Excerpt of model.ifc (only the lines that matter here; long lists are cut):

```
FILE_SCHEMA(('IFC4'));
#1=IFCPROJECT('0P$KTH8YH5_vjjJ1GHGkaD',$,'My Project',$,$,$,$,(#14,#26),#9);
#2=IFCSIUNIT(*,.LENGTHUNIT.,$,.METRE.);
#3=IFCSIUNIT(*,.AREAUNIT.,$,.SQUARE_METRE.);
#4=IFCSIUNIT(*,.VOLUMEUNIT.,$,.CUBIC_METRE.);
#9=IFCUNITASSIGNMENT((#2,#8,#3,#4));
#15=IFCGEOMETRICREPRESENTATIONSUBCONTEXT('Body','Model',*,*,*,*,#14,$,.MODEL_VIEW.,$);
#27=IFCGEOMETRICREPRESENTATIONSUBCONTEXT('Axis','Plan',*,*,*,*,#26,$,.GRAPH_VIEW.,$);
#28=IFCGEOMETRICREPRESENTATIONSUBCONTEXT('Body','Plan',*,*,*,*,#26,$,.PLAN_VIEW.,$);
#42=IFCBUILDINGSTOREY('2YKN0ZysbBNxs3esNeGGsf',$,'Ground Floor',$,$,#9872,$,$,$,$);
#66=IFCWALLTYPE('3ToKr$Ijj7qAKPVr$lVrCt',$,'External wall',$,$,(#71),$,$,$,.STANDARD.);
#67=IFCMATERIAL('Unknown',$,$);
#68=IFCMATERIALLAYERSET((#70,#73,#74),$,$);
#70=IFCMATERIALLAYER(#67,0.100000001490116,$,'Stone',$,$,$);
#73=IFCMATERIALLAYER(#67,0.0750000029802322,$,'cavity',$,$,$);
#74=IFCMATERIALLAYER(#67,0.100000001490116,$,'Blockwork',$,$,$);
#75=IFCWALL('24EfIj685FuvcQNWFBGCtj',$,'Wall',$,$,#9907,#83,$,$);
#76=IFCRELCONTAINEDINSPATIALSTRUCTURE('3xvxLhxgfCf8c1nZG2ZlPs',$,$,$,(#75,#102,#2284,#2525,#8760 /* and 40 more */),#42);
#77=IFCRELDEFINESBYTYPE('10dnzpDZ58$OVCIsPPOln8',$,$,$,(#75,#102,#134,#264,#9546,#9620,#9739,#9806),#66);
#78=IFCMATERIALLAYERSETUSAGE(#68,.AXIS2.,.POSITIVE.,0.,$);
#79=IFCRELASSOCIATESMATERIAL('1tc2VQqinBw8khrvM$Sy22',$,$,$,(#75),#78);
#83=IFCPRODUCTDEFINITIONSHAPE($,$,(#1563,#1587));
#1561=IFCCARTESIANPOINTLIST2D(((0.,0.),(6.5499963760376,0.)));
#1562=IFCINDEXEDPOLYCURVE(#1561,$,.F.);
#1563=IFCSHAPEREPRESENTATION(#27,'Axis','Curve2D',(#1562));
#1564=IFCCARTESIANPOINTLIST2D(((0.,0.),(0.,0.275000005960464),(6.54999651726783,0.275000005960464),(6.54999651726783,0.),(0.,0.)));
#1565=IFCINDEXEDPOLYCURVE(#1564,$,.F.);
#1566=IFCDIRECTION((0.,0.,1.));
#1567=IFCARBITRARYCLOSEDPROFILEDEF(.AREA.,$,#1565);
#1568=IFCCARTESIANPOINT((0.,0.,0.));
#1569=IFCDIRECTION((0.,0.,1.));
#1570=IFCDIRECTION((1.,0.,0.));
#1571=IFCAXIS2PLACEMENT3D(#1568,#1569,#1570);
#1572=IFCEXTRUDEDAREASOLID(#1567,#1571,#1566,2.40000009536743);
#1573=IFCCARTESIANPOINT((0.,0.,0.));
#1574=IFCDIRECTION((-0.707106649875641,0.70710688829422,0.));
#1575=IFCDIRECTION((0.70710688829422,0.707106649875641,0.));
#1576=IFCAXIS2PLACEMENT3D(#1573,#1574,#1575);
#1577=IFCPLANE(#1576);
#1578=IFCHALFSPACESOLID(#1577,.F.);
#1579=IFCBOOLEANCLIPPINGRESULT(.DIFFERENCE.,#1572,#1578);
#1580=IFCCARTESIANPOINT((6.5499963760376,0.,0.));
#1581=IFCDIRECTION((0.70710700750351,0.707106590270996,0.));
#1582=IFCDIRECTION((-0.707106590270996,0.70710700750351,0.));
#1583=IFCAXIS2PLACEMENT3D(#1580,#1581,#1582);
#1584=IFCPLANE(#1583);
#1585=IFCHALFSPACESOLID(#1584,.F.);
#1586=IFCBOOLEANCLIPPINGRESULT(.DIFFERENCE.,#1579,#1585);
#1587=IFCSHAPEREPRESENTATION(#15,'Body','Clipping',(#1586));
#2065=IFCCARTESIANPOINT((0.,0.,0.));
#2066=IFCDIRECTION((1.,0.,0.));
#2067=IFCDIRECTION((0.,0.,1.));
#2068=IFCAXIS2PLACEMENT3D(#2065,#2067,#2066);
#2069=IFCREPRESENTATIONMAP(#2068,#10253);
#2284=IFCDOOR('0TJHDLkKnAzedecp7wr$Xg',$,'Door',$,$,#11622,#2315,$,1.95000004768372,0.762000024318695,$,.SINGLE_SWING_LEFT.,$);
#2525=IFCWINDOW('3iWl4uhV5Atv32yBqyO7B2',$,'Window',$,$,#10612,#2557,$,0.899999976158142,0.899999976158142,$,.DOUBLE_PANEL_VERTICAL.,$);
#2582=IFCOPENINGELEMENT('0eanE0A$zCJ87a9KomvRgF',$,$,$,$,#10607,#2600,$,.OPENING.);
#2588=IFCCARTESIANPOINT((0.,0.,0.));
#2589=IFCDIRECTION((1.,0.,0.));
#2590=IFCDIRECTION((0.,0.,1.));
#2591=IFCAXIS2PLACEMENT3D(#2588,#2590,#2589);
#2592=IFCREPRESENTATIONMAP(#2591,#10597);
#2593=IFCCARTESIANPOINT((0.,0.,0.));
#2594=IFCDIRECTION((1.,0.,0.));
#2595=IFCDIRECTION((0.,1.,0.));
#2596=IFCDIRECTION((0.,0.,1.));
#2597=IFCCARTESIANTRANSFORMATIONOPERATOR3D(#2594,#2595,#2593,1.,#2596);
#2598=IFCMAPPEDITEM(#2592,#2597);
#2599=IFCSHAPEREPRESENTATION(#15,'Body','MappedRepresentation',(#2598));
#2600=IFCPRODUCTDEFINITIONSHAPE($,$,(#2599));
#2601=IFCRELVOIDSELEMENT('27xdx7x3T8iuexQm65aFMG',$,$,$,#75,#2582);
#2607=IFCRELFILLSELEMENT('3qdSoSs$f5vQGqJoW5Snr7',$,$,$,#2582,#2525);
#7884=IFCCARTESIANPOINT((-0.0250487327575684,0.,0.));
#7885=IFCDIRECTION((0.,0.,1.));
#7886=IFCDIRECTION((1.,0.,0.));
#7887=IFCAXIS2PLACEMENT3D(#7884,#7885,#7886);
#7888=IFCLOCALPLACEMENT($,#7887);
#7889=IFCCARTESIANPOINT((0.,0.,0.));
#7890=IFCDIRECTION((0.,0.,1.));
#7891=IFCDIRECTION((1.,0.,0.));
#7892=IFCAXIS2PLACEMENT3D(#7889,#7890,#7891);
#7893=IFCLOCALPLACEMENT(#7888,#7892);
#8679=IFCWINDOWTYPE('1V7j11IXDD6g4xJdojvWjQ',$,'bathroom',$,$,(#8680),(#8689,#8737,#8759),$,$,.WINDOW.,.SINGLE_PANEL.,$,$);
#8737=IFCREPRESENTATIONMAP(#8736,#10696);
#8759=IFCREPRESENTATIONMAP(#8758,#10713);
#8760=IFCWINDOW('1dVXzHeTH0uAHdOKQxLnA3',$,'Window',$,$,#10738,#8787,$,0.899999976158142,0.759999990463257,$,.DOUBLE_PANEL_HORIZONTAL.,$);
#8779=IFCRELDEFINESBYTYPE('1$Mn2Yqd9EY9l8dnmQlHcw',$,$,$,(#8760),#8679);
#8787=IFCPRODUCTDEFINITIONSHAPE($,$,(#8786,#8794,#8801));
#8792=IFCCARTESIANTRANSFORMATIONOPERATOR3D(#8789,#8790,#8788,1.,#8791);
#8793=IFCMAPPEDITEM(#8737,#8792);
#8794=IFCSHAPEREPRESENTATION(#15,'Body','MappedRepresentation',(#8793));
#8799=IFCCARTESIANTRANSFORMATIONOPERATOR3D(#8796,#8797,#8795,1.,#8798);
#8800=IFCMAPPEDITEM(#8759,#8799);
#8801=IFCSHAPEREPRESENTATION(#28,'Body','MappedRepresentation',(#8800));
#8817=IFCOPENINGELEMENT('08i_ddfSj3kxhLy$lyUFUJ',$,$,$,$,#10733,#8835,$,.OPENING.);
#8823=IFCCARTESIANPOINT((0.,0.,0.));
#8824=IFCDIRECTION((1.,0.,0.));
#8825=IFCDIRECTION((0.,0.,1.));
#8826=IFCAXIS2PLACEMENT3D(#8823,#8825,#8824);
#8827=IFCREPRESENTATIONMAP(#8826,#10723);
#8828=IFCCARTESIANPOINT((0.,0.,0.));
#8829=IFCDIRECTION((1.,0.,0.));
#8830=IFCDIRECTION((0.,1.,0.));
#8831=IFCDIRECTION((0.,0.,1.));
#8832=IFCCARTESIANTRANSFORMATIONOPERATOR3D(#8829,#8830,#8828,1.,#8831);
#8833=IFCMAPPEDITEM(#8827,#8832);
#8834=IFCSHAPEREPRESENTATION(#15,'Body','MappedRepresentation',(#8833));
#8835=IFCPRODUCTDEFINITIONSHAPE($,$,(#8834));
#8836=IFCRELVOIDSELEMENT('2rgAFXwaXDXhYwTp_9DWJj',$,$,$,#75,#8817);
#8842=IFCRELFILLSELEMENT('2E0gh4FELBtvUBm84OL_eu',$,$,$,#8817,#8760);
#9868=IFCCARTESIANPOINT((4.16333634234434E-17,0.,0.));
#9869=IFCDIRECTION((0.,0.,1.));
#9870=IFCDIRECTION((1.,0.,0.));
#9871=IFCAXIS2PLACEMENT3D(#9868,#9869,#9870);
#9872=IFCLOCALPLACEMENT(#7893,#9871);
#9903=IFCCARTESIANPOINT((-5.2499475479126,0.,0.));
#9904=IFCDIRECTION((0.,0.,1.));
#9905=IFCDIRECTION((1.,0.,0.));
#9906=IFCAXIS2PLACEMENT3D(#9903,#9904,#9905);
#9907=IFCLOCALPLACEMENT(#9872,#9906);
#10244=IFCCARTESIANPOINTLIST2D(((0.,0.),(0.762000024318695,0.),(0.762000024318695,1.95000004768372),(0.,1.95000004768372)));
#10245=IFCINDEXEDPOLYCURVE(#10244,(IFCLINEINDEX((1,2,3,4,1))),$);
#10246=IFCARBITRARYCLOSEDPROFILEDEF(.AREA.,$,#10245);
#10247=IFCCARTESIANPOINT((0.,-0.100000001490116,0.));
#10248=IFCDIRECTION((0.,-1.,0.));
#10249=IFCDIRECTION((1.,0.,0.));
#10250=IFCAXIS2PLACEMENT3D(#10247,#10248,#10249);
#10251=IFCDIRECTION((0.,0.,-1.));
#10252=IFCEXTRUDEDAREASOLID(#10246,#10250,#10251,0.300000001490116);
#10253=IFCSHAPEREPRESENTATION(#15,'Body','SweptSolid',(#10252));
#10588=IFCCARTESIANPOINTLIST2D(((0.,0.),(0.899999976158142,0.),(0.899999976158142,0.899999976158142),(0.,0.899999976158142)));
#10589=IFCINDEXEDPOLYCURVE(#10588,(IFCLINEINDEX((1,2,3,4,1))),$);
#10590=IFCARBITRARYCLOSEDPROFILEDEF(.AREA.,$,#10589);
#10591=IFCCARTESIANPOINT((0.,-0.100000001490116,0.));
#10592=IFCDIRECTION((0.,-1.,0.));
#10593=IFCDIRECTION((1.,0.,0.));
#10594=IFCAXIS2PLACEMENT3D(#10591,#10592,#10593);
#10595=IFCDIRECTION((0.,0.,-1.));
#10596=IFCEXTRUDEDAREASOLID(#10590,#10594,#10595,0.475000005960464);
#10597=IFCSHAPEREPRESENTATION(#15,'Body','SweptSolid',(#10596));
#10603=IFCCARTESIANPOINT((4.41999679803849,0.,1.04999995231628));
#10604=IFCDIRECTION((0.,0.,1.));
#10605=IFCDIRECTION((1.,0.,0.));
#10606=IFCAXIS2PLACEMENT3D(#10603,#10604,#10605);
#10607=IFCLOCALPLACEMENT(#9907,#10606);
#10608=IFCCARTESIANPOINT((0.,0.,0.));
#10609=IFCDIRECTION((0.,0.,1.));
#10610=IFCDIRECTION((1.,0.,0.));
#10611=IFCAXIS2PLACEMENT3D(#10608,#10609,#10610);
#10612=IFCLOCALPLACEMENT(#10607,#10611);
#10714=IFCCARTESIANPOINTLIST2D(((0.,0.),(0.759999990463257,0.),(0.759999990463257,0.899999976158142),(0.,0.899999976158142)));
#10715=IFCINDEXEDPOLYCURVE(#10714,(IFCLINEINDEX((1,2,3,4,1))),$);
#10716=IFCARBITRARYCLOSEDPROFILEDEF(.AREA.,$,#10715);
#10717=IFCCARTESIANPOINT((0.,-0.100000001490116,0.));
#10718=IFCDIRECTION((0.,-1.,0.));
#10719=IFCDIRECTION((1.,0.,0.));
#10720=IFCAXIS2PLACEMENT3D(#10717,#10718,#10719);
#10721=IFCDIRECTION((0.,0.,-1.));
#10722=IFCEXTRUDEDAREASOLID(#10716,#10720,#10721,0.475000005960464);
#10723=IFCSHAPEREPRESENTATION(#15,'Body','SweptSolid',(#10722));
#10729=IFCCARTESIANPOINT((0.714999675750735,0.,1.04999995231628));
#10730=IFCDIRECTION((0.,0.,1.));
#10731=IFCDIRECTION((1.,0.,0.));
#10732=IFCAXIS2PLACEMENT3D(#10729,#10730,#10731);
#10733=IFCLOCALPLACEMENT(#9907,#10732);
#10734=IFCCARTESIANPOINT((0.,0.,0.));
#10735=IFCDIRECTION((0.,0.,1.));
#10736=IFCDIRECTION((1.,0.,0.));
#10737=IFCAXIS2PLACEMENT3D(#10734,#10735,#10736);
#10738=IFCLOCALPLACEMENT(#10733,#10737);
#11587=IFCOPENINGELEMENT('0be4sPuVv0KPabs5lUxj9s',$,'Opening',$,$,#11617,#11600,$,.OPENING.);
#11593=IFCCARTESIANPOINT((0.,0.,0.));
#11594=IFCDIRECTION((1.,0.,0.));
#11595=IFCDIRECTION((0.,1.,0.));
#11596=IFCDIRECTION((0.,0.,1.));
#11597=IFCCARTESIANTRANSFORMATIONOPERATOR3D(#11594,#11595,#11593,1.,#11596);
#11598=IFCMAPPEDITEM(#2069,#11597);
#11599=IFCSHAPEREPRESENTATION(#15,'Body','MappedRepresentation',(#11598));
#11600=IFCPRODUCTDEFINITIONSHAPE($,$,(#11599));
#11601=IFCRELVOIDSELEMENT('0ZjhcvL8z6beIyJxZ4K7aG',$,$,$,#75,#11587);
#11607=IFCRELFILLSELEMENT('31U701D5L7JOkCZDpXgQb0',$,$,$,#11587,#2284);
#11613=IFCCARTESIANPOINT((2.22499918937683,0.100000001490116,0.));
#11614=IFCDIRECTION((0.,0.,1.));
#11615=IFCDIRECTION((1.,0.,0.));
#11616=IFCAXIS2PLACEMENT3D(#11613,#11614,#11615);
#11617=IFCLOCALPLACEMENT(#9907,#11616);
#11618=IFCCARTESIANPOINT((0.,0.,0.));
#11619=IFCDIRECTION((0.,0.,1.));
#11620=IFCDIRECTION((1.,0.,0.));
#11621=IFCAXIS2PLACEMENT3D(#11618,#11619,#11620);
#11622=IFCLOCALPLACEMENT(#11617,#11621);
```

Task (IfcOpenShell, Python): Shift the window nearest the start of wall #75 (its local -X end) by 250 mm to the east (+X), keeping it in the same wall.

```python
import ifcopenshell
import ifcopenshell.api.geometry
import ifcopenshell.util.placement
import ifcopenshell.util.unit

model = ifcopenshell.open("model.ifc")
unit_scale = ifcopenshell.util.unit.calculate_unit_scale(model)

window = model.by_id(8760)
opening = window.FillsVoids[0].RelatingOpeningElement
wall = opening.VoidsElements[0].RelatingBuildingElement

wall_matrix = ifcopenshell.util.placement.get_local_placement(wall.ObjectPlacement)
shift = wall_matrix[:3, 0] * 0.25 / unit_scale
before = ifcopenshell.util.placement.get_local_placement(window.ObjectPlacement)[:3, 3].copy()

# The window is placed relative to its opening, so it follows when the opening moves.
matrix = ifcopenshell.util.placement.get_local_placement(opening.ObjectPlacement)
matrix[:3, 3] += shift
ifcopenshell.api.geometry.edit_object_placement(
    model, product=opening, matrix=matrix, is_si=False, should_transform_children=True
)

after = ifcopenshell.util.placement.get_local_placement(window.ObjectPlacement)[:3, 3]
print("window moved by", (after - before).round(3) + 0.0)

model.write("model_rev.ifc")
```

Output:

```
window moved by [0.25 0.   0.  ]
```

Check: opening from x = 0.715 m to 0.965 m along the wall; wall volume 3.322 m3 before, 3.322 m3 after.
